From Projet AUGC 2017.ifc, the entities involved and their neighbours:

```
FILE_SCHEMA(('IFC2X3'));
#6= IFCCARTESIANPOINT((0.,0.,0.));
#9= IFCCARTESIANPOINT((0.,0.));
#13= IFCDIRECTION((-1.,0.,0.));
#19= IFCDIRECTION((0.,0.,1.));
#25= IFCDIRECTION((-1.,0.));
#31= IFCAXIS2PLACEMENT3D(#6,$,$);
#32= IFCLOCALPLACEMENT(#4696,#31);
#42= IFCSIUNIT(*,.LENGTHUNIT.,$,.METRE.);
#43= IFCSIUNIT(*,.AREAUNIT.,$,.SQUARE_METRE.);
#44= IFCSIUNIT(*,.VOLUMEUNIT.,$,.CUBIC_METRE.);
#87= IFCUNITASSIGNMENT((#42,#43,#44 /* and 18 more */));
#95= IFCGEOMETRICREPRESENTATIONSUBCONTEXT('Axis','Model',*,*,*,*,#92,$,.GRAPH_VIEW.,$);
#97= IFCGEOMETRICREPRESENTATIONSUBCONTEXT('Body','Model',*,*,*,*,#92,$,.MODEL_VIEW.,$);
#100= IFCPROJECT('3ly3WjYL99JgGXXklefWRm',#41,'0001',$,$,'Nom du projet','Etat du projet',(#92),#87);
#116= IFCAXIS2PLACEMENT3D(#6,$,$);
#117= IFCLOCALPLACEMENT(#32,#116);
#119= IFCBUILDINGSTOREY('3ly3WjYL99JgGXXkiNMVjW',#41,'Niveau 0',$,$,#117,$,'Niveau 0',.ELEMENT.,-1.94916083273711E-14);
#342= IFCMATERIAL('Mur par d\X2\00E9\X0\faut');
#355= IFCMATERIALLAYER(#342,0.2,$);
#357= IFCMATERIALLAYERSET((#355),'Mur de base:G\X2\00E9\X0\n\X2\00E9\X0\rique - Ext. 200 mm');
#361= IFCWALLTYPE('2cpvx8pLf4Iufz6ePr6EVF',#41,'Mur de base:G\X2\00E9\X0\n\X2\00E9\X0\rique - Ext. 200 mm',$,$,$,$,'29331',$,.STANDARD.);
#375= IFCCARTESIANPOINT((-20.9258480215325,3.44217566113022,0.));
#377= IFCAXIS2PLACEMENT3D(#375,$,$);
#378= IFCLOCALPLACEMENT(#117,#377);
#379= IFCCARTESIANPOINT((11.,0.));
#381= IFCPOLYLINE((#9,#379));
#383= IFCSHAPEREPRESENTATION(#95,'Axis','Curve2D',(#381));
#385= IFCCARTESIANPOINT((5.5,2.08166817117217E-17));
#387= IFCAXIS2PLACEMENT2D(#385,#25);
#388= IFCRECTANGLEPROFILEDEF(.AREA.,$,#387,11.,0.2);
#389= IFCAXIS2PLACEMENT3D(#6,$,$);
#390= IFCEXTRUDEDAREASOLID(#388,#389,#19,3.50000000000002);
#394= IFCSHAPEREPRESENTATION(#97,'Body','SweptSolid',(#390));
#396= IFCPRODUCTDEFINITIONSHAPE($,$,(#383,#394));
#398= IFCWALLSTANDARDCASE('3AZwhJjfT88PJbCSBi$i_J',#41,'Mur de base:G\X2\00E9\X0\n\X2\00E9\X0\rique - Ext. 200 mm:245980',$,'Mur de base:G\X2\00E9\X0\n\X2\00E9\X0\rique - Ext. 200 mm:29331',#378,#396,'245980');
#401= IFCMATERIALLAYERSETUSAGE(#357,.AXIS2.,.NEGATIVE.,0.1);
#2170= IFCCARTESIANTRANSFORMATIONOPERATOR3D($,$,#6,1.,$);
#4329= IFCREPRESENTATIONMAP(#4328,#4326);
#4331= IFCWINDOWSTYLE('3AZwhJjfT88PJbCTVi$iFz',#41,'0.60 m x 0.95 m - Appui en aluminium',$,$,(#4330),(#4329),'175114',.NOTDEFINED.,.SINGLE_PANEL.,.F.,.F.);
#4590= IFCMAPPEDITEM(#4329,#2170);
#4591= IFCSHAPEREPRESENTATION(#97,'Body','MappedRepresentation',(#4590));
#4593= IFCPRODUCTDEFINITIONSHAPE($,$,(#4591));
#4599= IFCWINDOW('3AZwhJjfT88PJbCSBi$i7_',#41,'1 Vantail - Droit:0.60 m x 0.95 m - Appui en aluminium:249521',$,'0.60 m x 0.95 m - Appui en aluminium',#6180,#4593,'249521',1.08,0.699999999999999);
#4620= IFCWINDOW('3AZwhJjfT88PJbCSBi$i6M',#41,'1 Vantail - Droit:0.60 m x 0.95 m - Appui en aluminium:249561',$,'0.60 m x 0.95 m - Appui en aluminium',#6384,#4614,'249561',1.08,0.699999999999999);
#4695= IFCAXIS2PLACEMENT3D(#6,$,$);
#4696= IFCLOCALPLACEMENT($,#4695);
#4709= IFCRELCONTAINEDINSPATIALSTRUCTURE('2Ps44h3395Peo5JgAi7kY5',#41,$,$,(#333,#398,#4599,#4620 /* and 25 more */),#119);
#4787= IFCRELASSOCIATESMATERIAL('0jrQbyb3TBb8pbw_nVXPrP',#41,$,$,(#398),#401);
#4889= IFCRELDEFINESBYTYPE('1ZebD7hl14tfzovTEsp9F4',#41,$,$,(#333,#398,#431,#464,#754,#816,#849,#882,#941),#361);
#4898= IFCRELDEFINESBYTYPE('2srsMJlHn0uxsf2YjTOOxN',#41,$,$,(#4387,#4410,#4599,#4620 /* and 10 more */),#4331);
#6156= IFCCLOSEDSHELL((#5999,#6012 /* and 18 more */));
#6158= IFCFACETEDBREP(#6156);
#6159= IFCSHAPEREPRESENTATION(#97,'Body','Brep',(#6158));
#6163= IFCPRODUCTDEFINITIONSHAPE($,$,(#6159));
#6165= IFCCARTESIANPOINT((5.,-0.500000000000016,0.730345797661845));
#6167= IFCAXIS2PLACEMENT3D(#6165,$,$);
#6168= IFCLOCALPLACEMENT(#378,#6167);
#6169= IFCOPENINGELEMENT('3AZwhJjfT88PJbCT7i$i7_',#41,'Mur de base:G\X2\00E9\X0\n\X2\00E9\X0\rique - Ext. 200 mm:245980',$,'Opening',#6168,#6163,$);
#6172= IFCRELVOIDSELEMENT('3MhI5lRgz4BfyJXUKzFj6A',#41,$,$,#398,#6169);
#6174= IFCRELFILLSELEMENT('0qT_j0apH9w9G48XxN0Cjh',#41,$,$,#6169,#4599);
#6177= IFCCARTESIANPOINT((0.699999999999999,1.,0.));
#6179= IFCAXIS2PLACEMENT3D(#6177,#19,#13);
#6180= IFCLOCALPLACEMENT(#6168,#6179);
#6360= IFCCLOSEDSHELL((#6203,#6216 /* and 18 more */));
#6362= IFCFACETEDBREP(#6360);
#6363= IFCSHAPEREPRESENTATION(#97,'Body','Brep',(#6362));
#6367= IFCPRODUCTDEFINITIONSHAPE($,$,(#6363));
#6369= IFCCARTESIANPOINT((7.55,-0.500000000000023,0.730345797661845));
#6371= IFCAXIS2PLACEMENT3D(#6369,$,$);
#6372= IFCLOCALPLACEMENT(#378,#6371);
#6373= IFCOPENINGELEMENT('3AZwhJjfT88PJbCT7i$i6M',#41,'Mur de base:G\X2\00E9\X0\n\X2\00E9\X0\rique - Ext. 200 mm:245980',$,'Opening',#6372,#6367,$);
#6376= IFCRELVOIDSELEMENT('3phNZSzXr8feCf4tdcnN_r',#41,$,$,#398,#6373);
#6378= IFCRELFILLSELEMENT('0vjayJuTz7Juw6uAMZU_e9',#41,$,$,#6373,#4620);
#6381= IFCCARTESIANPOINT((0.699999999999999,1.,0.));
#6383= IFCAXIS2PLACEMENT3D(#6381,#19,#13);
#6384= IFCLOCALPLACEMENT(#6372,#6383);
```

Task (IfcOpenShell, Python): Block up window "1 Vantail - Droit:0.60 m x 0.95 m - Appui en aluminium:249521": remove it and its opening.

```python
import ifcopenshell
import ifcopenshell.api.feature
import ifcopenshell.api.root
import ifcopenshell.geom
import ifcopenshell.util.shape

model = ifcopenshell.open("Projet AUGC 2017.ifc")
settings = ifcopenshell.geom.settings()


def volume(element):
    """Net volume in cubic metres, openings subtracted."""
    shape = ifcopenshell.geom.create_shape(settings, element)
    return ifcopenshell.util.shape.get_volume(shape.geometry)


window = model.by_id(4599)
opening = window.FillsVoids[0].RelatingOpeningElement
wall = opening.VoidsElements[0].RelatingBuildingElement
before = volume(wall)

ifcopenshell.api.root.remove_product(model, product=window)
ifcopenshell.api.feature.remove_feature(model, feature=opening)

after = volume(wall)

print(f"wall volume {before:.3f} -> {after:.3f} m3")

model.write("Projet AUGC 2017_updated.ifc")
```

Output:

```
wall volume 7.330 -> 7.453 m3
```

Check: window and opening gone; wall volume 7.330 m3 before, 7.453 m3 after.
